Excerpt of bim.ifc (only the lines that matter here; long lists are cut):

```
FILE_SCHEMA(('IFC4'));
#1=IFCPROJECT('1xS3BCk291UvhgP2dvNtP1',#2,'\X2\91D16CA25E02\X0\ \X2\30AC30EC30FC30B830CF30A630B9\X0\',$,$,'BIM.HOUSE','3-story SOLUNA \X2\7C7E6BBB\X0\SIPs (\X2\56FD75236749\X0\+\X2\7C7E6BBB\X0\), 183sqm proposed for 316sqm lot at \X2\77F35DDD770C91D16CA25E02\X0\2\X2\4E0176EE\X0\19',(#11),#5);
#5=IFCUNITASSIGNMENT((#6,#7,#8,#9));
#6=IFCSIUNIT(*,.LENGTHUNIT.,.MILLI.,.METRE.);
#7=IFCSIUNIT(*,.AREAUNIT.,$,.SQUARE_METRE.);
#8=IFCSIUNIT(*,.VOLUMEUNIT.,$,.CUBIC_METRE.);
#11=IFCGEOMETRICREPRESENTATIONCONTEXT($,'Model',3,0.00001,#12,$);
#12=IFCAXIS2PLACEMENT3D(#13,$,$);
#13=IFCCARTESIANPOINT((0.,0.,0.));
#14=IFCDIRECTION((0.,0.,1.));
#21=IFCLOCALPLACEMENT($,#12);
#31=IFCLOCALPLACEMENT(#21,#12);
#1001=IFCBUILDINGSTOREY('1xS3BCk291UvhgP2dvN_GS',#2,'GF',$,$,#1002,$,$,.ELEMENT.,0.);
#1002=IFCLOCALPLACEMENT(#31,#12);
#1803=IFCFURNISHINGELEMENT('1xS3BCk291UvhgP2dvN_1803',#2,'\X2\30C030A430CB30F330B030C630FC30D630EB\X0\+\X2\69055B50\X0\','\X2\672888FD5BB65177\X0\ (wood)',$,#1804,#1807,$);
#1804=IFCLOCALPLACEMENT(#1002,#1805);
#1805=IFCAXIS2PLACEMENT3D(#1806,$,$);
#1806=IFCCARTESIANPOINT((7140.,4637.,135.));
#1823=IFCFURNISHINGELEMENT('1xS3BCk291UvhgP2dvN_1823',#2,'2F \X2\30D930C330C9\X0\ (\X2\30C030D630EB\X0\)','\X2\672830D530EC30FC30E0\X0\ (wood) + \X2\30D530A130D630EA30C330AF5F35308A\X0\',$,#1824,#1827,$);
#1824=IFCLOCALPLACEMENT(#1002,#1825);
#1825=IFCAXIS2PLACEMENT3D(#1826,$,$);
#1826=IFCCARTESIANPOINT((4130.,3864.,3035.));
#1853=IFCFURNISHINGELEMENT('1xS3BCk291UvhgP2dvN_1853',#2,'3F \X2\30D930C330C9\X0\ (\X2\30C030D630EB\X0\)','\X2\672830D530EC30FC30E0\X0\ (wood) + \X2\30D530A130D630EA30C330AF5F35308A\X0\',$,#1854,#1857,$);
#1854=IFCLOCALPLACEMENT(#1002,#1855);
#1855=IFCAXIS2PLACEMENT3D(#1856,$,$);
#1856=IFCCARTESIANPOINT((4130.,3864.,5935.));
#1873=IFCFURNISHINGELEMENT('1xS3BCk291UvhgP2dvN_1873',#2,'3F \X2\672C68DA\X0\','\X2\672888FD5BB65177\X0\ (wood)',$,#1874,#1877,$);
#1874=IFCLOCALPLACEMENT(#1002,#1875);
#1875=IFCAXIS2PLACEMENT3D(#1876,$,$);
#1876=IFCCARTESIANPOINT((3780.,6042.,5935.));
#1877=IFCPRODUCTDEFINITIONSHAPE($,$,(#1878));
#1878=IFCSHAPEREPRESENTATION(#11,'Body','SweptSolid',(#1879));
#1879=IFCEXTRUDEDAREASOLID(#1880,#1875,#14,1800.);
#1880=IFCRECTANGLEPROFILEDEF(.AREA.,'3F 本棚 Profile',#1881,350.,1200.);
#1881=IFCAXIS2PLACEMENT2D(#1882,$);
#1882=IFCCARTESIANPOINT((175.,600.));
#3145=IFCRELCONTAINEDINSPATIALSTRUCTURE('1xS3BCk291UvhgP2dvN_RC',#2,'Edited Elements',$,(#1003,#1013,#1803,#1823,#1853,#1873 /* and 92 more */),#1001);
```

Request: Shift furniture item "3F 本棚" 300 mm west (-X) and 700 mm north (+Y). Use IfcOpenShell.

```python
import ifcopenshell
import ifcopenshell.api.geometry
import ifcopenshell.util.placement

model = ifcopenshell.open("bim.ifc")

item = model.by_guid("1xS3BCk291UvhgP2dvN_1873")
matrix = ifcopenshell.util.placement.get_local_placement(item.ObjectPlacement)
matrix[0, 3] -= 300.0
matrix[1, 3] += 700.0
ifcopenshell.api.geometry.edit_object_placement(model, product=item, matrix=matrix, is_si=False)

print(ifcopenshell.util.placement.get_local_placement(item.ObjectPlacement).round(3) + 0.0)

model.write("bim_rev.ifc")
```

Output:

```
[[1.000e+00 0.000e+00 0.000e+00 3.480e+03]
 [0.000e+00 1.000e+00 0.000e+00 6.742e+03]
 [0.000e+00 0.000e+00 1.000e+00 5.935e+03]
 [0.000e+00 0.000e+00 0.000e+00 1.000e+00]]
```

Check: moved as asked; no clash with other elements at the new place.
